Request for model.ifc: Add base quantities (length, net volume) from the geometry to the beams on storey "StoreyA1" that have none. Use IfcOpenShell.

First a look at what the model holds.

```python
import ifcopenshell
import ifcopenshell.util.element
import ifcopenshell.util.unit

model = ifcopenshell.open("model.ifc")
print(model.schema)
for unit_type in ("LENGTHUNIT", "AREAUNIT", "VOLUMEUNIT"):
    print(unit_type, ifcopenshell.util.unit.calculate_unit_scale(model, unit_type))
storey = next(s for s in model.by_type("IfcBuildingStorey") if s.Name == "StoreyA1")
beams = [e for e in ifcopenshell.util.element.get_decomposition(storey) if e.is_a("IfcBeam")]
for e in sorted(beams, key=lambda e: e.id()):
    print(e.id(), e.is_a(), e.Name, list(ifcopenshell.util.element.get_psets(e, qtos_only=True)), sep=" | ")
```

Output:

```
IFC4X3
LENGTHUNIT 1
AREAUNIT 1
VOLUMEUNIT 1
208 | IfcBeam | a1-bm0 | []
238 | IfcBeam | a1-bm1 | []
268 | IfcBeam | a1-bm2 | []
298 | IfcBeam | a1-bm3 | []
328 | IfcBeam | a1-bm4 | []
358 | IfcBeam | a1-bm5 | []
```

```python
import ifcopenshell
import ifcopenshell.api.pset
import ifcopenshell.geom
import ifcopenshell.util.element
import ifcopenshell.util.shape
import ifcopenshell.util.unit

model = ifcopenshell.open("model.ifc")
unit_scale = ifcopenshell.util.unit.calculate_unit_scale(model)
volume_scale = ifcopenshell.util.unit.calculate_unit_scale(model, "VOLUMEUNIT")
settings = ifcopenshell.geom.settings()

storey = next(s for s in model.by_type("IfcBuildingStorey") if s.Name == "StoreyA1")
beams = [e for e in ifcopenshell.util.element.get_decomposition(storey) if e.is_a("IfcBeam")]

for e in sorted(beams, key=lambda e: e.id()):
    if ifcopenshell.util.element.get_psets(e, qtos_only=True, should_inherit=False):
        continue
    # Geometry comes back in metres, in the element's own axes.
    shape = ifcopenshell.geom.create_shape(settings, e)
    values = {
        "Length": ifcopenshell.util.shape.get_max_xyz(shape.geometry) / unit_scale,
        "NetVolume": ifcopenshell.util.shape.get_volume(shape.geometry) / volume_scale,
    }
    qto = ifcopenshell.api.pset.add_qto(model, product=e, name="Qto_BeamBaseQuantities")
    ifcopenshell.api.pset.edit_qto(model, qto=qto, properties=values)
    print(e.id(), {k: round(v, 3) for k, v in values.items()})

model.write("model_rev.ifc")
```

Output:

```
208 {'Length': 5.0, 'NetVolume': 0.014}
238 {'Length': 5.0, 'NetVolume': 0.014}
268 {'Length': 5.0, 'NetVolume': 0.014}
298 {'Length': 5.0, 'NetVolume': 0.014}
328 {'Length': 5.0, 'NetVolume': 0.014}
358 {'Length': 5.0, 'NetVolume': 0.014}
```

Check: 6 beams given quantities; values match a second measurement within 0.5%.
